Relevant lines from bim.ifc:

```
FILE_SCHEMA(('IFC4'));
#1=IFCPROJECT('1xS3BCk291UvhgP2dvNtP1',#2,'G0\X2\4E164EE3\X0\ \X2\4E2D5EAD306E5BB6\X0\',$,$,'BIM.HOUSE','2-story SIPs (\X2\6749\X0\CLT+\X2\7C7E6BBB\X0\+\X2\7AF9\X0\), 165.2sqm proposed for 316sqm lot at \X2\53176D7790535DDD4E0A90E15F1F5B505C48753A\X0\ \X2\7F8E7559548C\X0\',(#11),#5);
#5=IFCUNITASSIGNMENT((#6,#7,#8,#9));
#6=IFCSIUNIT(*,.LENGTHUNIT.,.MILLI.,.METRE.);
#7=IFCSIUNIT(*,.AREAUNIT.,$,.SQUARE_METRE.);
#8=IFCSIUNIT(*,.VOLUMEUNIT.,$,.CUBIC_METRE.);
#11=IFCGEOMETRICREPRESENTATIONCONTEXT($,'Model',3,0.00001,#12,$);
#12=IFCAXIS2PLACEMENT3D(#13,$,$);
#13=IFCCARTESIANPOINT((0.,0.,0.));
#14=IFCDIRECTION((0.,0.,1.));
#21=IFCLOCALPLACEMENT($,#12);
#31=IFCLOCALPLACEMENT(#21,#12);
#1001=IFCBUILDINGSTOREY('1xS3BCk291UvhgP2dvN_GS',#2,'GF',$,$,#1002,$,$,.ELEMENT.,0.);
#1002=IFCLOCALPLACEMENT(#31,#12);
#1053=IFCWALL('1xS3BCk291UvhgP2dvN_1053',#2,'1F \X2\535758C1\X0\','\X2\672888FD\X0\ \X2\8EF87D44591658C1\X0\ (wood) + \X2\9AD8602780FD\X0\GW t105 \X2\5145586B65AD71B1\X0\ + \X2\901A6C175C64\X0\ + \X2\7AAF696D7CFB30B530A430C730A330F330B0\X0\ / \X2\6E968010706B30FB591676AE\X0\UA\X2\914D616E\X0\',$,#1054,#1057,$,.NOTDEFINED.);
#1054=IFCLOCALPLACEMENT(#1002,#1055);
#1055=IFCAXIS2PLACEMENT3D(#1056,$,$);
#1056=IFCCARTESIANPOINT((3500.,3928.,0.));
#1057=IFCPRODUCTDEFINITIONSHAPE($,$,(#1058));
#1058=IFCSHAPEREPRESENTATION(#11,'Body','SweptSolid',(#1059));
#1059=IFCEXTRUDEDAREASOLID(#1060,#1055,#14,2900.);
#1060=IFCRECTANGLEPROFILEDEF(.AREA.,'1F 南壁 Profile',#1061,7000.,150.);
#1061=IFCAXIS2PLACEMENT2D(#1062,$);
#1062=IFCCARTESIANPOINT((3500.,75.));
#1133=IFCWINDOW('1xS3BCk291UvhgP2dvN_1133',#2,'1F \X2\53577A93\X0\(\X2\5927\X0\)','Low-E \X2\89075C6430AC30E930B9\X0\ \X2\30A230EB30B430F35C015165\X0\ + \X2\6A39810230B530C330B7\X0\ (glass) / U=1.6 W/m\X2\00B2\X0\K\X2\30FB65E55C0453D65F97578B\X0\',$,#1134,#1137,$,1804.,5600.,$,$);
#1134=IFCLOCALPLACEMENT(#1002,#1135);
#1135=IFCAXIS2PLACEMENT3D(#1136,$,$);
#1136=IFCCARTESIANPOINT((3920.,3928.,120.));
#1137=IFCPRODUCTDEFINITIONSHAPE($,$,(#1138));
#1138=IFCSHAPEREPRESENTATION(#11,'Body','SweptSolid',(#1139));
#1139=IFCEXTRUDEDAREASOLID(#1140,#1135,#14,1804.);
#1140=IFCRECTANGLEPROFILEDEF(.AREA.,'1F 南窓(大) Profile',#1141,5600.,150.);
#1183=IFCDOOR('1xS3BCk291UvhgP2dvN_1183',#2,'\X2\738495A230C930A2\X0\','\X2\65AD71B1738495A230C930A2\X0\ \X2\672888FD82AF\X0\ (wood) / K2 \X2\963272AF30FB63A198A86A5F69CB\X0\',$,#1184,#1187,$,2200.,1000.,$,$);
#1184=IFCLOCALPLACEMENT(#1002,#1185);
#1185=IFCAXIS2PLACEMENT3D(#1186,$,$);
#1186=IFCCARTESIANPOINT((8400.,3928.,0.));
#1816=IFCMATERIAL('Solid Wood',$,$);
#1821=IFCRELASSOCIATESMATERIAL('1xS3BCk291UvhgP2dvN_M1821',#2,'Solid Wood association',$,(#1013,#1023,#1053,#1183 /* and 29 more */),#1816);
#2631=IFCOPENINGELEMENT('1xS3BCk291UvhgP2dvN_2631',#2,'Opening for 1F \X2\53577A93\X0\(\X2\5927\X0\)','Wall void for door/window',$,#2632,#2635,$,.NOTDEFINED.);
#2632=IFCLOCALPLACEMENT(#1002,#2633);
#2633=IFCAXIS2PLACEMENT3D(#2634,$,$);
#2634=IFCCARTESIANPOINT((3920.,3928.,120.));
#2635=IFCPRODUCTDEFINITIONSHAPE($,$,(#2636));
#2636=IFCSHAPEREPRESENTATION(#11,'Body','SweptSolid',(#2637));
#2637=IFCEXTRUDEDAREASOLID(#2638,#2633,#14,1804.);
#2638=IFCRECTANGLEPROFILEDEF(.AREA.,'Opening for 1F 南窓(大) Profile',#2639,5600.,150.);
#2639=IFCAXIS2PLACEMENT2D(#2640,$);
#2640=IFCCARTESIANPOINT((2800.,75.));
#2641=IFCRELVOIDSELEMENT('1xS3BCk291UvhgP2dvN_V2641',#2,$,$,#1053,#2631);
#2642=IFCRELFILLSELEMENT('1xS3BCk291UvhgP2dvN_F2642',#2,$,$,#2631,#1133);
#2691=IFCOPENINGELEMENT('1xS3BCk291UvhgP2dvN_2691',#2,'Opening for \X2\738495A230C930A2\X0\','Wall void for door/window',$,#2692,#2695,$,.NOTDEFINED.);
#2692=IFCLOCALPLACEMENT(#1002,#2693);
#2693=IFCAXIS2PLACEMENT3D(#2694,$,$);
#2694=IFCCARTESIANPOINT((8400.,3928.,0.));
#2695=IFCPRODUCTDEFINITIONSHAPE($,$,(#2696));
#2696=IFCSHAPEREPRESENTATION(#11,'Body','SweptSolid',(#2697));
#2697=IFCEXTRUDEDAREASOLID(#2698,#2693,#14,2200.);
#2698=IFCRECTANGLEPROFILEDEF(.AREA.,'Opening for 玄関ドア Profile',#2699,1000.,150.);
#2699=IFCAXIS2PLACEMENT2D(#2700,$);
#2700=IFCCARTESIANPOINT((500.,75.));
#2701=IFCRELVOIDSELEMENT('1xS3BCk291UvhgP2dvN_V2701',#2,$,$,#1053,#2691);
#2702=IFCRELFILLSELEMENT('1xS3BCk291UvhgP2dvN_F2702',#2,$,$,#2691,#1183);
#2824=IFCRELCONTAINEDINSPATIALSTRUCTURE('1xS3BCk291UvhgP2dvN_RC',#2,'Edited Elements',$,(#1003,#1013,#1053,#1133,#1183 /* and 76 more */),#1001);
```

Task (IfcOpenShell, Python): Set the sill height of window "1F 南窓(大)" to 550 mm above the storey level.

```python
import numpy as np
import ifcopenshell
import ifcopenshell.api.geometry
import ifcopenshell.geom
import ifcopenshell.util.element
import ifcopenshell.util.placement
import ifcopenshell.util.shape
import ifcopenshell.util.unit

model = ifcopenshell.open("bim.ifc")
unit_scale = ifcopenshell.util.unit.calculate_unit_scale(model)

window = model.by_guid("1xS3BCk291UvhgP2dvN_1133")
opening = window.FillsVoids[0].RelatingOpeningElement
storey = ifcopenshell.util.element.get_container(window, ifc_class="IfcBuildingStorey")
level = ifcopenshell.util.placement.get_local_placement(storey.ObjectPlacement)[2, 3]

# The opening's origin need not be at the sill, so measure its lowest point.
shape = ifcopenshell.geom.create_shape(ifcopenshell.geom.settings(), opening)
bottom = ifcopenshell.util.shape.get_shape_bottom_elevation(shape, shape.geometry) / unit_scale
dz = level + 550.0 - bottom

shift = np.array([0.0, 0.0, dz])
# The window is not placed relative to its opening, so move both.
for product in (opening, window):
    matrix = ifcopenshell.util.placement.get_local_placement(product.ObjectPlacement)
    matrix[:3, 3] += shift
    ifcopenshell.api.geometry.edit_object_placement(model, product=product, matrix=matrix, is_si=False)

print(f"moved by {dz * unit_scale:+.3f} m")

model.write("bim_updated.ifc")
```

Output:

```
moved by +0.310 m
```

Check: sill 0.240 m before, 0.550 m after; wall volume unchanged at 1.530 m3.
